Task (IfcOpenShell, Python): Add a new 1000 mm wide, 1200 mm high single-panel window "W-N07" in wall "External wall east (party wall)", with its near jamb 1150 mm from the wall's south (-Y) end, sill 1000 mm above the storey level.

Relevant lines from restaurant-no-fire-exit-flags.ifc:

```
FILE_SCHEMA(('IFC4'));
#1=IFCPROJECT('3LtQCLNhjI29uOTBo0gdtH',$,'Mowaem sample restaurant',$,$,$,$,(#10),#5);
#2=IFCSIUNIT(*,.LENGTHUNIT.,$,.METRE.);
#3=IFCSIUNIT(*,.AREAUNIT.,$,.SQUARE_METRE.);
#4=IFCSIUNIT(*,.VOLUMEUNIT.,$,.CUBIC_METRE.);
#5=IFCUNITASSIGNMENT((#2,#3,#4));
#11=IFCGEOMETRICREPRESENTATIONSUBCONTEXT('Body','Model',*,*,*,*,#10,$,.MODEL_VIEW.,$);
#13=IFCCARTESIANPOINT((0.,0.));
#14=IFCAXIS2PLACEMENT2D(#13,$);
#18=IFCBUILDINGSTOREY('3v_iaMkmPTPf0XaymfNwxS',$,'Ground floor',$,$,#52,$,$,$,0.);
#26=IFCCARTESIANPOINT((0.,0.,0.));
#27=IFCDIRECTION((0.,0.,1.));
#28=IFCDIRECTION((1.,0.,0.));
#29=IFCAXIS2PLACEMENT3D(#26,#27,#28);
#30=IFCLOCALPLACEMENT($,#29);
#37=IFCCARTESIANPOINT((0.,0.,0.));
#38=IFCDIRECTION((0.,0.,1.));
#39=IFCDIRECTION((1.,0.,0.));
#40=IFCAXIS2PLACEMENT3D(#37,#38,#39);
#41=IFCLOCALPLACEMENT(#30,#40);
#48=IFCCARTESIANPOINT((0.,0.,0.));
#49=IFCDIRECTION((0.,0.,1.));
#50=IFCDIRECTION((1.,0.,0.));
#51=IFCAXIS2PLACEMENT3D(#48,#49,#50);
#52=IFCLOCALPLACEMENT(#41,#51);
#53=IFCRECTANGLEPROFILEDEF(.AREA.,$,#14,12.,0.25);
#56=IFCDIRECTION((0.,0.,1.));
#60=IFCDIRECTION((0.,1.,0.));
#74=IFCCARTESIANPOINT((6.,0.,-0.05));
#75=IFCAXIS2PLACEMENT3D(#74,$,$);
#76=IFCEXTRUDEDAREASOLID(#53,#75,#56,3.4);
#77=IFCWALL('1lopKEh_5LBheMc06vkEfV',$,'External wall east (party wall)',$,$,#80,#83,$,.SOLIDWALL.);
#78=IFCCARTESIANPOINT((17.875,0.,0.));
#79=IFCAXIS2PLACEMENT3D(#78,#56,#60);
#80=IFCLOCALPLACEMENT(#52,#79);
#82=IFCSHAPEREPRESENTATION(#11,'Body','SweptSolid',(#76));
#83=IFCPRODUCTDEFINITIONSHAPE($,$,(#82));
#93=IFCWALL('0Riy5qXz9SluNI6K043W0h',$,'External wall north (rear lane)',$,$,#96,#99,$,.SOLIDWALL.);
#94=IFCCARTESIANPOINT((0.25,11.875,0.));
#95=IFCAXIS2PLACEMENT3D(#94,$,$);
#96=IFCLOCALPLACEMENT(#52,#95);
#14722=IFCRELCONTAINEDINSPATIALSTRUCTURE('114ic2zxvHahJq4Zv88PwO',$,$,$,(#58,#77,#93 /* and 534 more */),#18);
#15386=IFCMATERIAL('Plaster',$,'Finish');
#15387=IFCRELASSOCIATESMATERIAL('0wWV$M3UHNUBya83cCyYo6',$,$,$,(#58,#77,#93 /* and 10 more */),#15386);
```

```python
import numpy as np
import ifcopenshell
import ifcopenshell.api.feature
import ifcopenshell.api.geometry
import ifcopenshell.api.root
import ifcopenshell.api.spatial
import ifcopenshell.geom
import ifcopenshell.util.element
import ifcopenshell.util.placement
import ifcopenshell.util.representation
import ifcopenshell.util.shape
import ifcopenshell.util.unit

model = ifcopenshell.open("restaurant-no-fire-exit-flags.ifc")
unit_scale = ifcopenshell.util.unit.calculate_unit_scale(model)
settings = ifcopenshell.geom.settings()


def volume(element):
    """Net volume in cubic metres, openings subtracted."""
    shape = ifcopenshell.geom.create_shape(settings, element)
    return ifcopenshell.util.shape.get_volume(shape.geometry)


wall = model.by_id(77)
storey = ifcopenshell.util.element.get_container(wall, ifc_class="IfcBuildingStorey")
context = ifcopenshell.util.representation.get_context(model, "Model", "Body", "MODEL_VIEW")
before = volume(wall)

width, height, from_end, sill = 1, 1.2, 1.15, 1  # metres

# The wall runs along its own X axis, and the end named is its -X end.
wall_shape = ifcopenshell.geom.create_shape(settings, wall)
x, y, z = ifcopenshell.util.shape.get_vertices(wall_shape.geometry).T
start = x.min() + from_end
face, thickness = float(y.min()), float(y.max() - y.min())
wall_matrix = ifcopenshell.util.placement.get_local_placement(wall.ObjectPlacement)
level = ifcopenshell.util.placement.get_local_placement(storey.ObjectPlacement)[2, 3]


def in_wall(x, y):
    """Placement at x, y metres in the wall's axes, at sill height."""
    matrix = wall_matrix.copy()
    matrix[:, 3] = wall_matrix @ np.array([x / unit_scale, y / unit_scale, 0.0, 1.0])
    matrix[2, 3] = level + sill / unit_scale
    return matrix


# Opening: a box that overshoots both wall faces by 50 mm.
opening = ifcopenshell.api.root.create_entity(model, ifc_class="IfcOpeningElement", predefined_type="OPENING")
box = ifcopenshell.api.geometry.add_wall_representation(
    model, context=context, length=width, height=height, thickness=thickness + 0.1
)
ifcopenshell.api.geometry.assign_representation(model, product=opening, representation=box)
ifcopenshell.api.geometry.edit_object_placement(model, product=opening, matrix=in_wall(start, face - 0.05), is_si=False)
ifcopenshell.api.feature.add_feature(model, feature=opening, element=wall)

window = ifcopenshell.api.root.create_entity(model, ifc_class="IfcWindow", name="W-N07", predefined_type="WINDOW")
window.OverallWidth, window.OverallHeight = width / unit_scale, height / unit_scale
window.PartitioningType = "SINGLE_PANEL"
body = ifcopenshell.api.geometry.add_window_representation(
    model,
    context=context,
    overall_width=window.OverallWidth,
    overall_height=window.OverallHeight,
    partition_type="SINGLE_PANEL",
)
ifcopenshell.api.geometry.assign_representation(model, product=window, representation=body)
ifcopenshell.api.spatial.assign_container(model, products=[window], relating_structure=storey)
ifcopenshell.api.feature.add_filling(model, opening=opening, element=window)

# Centre the window in the wall's thickness.
ifcopenshell.api.geometry.edit_object_placement(model, product=window, matrix=in_wall(start, face), is_si=False)
window_shape = ifcopenshell.geom.create_shape(settings, window)
depth = ifcopenshell.util.shape.get_vertices(window_shape.geometry)[:, 1]
offset = face + thickness / 2 - (depth.min() + depth.max()) / 2
ifcopenshell.api.geometry.edit_object_placement(model, product=window, matrix=in_wall(start, offset), is_si=False)

after = volume(wall)

print(f"wall volume {before:.3f} -> {after:.3f} m3")

model.write("restaurant-no-fire-exit-flags_edited.ifc")
```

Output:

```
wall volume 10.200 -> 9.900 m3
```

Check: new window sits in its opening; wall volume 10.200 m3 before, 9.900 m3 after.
